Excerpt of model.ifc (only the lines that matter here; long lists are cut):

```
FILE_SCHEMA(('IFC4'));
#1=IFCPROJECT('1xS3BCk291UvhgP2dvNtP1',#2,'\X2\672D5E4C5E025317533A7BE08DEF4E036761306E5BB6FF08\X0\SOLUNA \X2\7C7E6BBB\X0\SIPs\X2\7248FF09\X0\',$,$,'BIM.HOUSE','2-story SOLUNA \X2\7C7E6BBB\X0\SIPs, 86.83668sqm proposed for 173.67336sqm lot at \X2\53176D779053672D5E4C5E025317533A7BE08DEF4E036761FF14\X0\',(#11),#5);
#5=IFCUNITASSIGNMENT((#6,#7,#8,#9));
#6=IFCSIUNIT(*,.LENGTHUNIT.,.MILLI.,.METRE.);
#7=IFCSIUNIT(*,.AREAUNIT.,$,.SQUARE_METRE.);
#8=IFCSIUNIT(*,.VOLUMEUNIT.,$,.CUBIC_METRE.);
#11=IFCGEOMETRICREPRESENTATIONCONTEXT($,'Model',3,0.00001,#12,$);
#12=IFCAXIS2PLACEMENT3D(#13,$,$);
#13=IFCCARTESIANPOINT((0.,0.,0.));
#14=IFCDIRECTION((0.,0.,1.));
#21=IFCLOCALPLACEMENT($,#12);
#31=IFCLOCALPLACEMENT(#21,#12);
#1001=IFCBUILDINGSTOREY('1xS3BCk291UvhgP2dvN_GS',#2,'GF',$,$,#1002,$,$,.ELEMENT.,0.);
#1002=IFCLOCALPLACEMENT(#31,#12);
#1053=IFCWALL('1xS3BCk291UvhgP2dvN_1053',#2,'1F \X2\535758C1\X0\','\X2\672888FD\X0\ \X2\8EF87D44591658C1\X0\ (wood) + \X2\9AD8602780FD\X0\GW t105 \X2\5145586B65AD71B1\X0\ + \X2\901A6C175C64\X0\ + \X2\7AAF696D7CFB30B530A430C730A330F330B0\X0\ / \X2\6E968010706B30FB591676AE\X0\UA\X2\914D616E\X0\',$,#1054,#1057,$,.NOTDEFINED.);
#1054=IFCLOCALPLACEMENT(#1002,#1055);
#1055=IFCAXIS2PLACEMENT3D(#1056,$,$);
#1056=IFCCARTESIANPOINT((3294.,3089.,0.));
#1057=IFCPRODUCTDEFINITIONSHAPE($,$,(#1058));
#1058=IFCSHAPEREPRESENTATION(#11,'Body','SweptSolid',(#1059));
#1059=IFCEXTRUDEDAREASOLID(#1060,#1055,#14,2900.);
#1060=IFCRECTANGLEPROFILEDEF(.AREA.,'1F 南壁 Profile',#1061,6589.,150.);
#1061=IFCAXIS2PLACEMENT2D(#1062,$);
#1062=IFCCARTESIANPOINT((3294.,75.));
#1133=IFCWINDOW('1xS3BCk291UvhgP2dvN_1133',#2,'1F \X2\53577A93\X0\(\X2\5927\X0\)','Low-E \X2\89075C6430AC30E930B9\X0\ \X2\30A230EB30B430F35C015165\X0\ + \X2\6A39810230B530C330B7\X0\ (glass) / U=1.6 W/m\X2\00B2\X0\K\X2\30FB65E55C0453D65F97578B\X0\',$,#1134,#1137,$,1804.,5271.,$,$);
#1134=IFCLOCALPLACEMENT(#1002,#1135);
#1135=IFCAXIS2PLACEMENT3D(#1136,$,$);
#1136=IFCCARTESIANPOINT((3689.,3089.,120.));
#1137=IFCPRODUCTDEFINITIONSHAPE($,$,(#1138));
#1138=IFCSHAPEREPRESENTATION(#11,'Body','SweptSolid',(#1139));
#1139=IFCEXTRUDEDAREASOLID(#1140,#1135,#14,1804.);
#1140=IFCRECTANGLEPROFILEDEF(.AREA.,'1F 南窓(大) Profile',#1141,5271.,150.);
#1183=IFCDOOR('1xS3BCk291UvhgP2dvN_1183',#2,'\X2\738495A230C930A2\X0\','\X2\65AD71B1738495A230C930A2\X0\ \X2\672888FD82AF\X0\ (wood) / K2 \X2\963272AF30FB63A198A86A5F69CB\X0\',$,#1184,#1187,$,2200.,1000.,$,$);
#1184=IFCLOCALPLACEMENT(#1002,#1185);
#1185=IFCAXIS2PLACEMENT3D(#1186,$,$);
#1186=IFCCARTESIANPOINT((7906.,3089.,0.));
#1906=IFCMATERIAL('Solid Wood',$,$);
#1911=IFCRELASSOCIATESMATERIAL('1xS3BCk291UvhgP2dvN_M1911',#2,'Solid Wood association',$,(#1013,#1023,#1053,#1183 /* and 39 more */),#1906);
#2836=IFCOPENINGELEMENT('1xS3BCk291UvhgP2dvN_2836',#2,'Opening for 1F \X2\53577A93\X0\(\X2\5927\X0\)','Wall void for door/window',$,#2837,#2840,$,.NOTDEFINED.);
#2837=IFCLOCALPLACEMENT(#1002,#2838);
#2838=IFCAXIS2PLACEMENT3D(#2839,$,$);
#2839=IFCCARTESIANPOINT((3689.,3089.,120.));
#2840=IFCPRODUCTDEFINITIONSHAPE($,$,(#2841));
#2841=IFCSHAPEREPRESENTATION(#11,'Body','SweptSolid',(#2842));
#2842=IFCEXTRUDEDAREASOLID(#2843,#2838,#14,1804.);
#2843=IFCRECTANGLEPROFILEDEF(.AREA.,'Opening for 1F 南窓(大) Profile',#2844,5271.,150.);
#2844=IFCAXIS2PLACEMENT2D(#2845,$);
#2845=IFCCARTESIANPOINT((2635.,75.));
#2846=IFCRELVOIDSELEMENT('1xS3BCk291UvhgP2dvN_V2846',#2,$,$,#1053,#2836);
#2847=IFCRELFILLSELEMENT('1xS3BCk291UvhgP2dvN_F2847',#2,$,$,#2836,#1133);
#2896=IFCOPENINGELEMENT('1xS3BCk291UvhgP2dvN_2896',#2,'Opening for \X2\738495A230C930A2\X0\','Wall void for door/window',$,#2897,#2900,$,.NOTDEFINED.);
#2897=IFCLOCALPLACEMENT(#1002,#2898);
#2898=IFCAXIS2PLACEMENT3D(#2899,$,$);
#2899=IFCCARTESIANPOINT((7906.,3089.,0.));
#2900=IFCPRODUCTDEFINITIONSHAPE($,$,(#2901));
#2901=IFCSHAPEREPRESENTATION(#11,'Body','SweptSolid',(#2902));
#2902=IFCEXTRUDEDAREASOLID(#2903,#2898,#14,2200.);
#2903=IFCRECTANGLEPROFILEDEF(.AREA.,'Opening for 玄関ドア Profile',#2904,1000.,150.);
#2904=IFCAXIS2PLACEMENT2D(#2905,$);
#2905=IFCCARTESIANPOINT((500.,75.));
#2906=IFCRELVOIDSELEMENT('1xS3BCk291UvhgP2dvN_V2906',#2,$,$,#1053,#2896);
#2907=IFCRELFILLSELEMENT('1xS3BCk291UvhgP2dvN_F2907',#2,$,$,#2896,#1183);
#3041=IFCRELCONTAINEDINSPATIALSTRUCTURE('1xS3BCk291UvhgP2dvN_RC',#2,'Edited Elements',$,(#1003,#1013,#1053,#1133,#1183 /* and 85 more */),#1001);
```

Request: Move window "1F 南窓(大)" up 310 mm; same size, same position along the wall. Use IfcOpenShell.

```python
import numpy as np
import ifcopenshell
import ifcopenshell.api.geometry
import ifcopenshell.util.placement
import ifcopenshell.util.unit

model = ifcopenshell.open("model.ifc")
unit_scale = ifcopenshell.util.unit.calculate_unit_scale(model)

window = model.by_guid("1xS3BCk291UvhgP2dvN_1133")
opening = window.FillsVoids[0].RelatingOpeningElement
dz = 310.0

shift = np.array([0.0, 0.0, dz])
# The window is not placed relative to its opening, so move both.
for product in (opening, window):
    matrix = ifcopenshell.util.placement.get_local_placement(product.ObjectPlacement)
    matrix[:3, 3] += shift
    ifcopenshell.api.geometry.edit_object_placement(model, product=product, matrix=matrix, is_si=False)

print(f"moved by {dz * unit_scale:+.3f} m")

model.write("model_v2.ifc")
```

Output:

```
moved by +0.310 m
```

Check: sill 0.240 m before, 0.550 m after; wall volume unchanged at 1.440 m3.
